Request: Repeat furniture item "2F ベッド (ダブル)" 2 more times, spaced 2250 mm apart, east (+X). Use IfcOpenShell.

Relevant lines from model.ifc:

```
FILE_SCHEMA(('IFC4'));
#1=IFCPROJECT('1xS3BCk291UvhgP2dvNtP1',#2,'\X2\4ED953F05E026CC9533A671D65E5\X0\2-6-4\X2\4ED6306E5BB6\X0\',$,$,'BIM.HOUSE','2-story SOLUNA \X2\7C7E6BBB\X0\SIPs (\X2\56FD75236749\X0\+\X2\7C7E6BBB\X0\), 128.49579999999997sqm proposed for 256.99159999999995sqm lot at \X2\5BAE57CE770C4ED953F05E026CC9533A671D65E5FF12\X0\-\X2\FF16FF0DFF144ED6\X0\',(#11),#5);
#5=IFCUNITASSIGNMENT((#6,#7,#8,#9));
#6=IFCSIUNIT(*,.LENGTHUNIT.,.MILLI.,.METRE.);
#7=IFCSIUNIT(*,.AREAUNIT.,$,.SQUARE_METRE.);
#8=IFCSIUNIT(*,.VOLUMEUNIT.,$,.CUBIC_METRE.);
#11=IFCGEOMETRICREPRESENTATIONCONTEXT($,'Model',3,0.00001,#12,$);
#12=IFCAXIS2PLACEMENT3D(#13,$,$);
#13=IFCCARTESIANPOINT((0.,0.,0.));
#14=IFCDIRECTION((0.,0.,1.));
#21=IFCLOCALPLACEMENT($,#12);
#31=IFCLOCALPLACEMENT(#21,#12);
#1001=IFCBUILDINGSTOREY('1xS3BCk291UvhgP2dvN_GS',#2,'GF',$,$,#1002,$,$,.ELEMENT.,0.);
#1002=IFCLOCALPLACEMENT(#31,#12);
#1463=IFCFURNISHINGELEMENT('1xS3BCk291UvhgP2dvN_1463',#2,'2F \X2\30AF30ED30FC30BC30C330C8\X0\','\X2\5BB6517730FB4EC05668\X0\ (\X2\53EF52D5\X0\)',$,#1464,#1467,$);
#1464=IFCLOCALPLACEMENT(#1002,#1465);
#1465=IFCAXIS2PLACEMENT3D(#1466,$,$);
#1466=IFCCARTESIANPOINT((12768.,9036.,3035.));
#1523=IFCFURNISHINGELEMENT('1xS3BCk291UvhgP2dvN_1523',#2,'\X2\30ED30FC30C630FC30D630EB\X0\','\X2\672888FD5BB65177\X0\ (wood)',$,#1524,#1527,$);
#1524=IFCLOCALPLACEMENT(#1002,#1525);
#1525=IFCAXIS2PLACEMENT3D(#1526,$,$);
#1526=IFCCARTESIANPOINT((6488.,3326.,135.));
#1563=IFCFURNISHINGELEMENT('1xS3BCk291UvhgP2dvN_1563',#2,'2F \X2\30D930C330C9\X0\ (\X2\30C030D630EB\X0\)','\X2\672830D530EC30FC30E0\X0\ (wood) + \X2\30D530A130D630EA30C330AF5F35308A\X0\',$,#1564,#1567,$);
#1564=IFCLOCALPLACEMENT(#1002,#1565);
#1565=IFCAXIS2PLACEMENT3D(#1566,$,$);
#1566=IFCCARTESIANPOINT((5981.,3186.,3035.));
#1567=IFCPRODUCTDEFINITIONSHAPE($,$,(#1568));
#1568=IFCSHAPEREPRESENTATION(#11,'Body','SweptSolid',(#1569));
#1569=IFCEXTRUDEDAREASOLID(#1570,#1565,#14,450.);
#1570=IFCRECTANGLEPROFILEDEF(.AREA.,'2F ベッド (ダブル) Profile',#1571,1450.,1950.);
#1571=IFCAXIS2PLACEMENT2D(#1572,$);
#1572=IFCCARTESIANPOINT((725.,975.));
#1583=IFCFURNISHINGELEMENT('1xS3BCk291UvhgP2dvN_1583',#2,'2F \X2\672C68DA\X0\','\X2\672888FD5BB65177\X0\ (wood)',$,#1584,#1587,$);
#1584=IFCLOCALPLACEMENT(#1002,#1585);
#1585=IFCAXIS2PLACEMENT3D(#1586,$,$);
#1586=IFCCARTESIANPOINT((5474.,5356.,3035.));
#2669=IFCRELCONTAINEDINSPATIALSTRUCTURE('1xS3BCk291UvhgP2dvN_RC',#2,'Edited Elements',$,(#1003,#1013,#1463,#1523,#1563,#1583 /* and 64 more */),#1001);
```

```python
import numpy as np
import ifcopenshell
import ifcopenshell.api.geometry
import ifcopenshell.api.root
import ifcopenshell.util.element
import ifcopenshell.util.placement

model = ifcopenshell.open("model.ifc")


def reuse_history(source, copy):
    """copy_class also copies each property set's owner history, people and application; keep the originals."""
    for rel in copy.IsDefinedBy:
        if rel.is_a("IfcRelDefinesByProperties") and (history := rel.RelatingPropertyDefinition.OwnerHistory):
            rel.RelatingPropertyDefinition.OwnerHistory = source.OwnerHistory
            ifcopenshell.util.element.remove_deep2(model, history)


source = model.by_guid("1xS3BCk291UvhgP2dvN_1563")
base = ifcopenshell.util.placement.get_local_placement(source.ObjectPlacement)
step = np.array([1.0, 0.0, 0.0]) * 2250.0

for i in range(1, 3):
    copy = ifcopenshell.api.root.copy_class(model, product=source)
    copy.Representation = ifcopenshell.util.element.copy_deep(
        model, source.Representation, exclude=["IfcGeometricRepresentationContext", "IfcRepresentationMap"]
    )
    reuse_history(source, copy)
    matrix = base.copy()
    matrix[:3, 3] += i * step
    print("added at", matrix[:3, 3].round(3) + 0.0)
    ifcopenshell.api.geometry.edit_object_placement(model, product=copy, matrix=matrix, is_si=False)

model.write("model-out.ifc")
```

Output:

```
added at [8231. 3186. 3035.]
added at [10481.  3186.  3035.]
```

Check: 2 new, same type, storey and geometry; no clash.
